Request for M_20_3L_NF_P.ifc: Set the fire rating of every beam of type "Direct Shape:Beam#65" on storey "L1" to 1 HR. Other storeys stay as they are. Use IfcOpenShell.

First a look at what the model holds.

```python
import ifcopenshell
import ifcopenshell.util.element

model = ifcopenshell.open("M_20_3L_NF_P.ifc")
print(model.schema)
storey = next(s for s in model.by_type("IfcBuildingStorey") if s.Name == "L1")
beams = [e for e in ifcopenshell.util.element.get_decomposition(storey) if e.is_a("IfcBeam")]
seen = {}
for e in beams:
    element_type = ifcopenshell.util.element.get_type(e)
    key = (element_type.Name if element_type != e and element_type else None, ifcopenshell.util.element.get_pset(e, "Pset_BeamCommon", "FireRating"))
    seen[key] = seen.get(key, 0) + 1
for (name, value), count in sorted(seen.items(), key=str):
    print(count, "x", name, "|", value)
```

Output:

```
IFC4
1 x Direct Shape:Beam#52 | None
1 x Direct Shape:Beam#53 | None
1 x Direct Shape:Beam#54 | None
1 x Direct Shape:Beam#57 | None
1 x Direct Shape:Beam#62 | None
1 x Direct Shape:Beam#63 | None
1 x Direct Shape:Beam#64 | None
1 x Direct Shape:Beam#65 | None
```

```python
import ifcopenshell
import ifcopenshell.api.pset
import ifcopenshell.util.element

model = ifcopenshell.open("M_20_3L_NF_P.ifc")

storey = next(s for s in model.by_type("IfcBuildingStorey") if s.Name == "L1")
beams = [e for e in ifcopenshell.util.element.get_decomposition(storey) if e.is_a("IfcBeam")]

count = 0
for e in beams:
    element_type = ifcopenshell.util.element.get_type(e)
    if element_type in (None, e) or element_type.Name != "Direct Shape:Beam#65":
        continue
    # add_pset returns the element's existing set when there is one.
    pset = ifcopenshell.api.pset.add_pset(model, product=e, name="Pset_BeamCommon")
    ifcopenshell.api.pset.edit_pset(model, pset=pset, properties={"FireRating": "1 HR"})
    count += 1

print(count, "beams updated")

model.write("M_20_3L_NF_P_edited.ifc")
```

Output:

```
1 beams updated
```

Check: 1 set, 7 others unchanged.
